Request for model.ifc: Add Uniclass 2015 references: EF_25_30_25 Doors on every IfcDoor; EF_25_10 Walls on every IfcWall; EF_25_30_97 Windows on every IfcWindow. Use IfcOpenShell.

First a look at what the model holds.

```python
import ifcopenshell

model = ifcopenshell.open("model.ifc")
print(model.schema)
print("classifications:", [c.Name for c in model.by_type("IfcClassification")])
for ifc_class in ("IfcDoor", "IfcRoof", "IfcStair", "IfcWall", "IfcWindow"):
    print(ifc_class, len(model.by_type(ifc_class)))
```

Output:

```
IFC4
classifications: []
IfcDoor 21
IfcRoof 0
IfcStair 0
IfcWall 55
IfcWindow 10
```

```python
import ifcopenshell
import ifcopenshell.api.classification

model = ifcopenshell.open("model.ifc")

system = ifcopenshell.api.classification.add_classification(model, classification="Uniclass 2015")

codes = {
    "IfcDoor": ("EF_25_30_25", "Doors"),
    "IfcWall": ("EF_25_10", "Walls"),
    "IfcWindow": ("EF_25_30_97", "Windows"),
}
for ifc_class, (code, name) in codes.items():
    products = model.by_type(ifc_class)
    ifcopenshell.api.classification.add_reference(
        model, products=products, classification=system, identification=code, name=name
    )
    print(code, len(products))

model.write("model_v2.ifc")
```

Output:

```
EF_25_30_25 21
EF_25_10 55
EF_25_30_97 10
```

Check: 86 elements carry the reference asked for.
